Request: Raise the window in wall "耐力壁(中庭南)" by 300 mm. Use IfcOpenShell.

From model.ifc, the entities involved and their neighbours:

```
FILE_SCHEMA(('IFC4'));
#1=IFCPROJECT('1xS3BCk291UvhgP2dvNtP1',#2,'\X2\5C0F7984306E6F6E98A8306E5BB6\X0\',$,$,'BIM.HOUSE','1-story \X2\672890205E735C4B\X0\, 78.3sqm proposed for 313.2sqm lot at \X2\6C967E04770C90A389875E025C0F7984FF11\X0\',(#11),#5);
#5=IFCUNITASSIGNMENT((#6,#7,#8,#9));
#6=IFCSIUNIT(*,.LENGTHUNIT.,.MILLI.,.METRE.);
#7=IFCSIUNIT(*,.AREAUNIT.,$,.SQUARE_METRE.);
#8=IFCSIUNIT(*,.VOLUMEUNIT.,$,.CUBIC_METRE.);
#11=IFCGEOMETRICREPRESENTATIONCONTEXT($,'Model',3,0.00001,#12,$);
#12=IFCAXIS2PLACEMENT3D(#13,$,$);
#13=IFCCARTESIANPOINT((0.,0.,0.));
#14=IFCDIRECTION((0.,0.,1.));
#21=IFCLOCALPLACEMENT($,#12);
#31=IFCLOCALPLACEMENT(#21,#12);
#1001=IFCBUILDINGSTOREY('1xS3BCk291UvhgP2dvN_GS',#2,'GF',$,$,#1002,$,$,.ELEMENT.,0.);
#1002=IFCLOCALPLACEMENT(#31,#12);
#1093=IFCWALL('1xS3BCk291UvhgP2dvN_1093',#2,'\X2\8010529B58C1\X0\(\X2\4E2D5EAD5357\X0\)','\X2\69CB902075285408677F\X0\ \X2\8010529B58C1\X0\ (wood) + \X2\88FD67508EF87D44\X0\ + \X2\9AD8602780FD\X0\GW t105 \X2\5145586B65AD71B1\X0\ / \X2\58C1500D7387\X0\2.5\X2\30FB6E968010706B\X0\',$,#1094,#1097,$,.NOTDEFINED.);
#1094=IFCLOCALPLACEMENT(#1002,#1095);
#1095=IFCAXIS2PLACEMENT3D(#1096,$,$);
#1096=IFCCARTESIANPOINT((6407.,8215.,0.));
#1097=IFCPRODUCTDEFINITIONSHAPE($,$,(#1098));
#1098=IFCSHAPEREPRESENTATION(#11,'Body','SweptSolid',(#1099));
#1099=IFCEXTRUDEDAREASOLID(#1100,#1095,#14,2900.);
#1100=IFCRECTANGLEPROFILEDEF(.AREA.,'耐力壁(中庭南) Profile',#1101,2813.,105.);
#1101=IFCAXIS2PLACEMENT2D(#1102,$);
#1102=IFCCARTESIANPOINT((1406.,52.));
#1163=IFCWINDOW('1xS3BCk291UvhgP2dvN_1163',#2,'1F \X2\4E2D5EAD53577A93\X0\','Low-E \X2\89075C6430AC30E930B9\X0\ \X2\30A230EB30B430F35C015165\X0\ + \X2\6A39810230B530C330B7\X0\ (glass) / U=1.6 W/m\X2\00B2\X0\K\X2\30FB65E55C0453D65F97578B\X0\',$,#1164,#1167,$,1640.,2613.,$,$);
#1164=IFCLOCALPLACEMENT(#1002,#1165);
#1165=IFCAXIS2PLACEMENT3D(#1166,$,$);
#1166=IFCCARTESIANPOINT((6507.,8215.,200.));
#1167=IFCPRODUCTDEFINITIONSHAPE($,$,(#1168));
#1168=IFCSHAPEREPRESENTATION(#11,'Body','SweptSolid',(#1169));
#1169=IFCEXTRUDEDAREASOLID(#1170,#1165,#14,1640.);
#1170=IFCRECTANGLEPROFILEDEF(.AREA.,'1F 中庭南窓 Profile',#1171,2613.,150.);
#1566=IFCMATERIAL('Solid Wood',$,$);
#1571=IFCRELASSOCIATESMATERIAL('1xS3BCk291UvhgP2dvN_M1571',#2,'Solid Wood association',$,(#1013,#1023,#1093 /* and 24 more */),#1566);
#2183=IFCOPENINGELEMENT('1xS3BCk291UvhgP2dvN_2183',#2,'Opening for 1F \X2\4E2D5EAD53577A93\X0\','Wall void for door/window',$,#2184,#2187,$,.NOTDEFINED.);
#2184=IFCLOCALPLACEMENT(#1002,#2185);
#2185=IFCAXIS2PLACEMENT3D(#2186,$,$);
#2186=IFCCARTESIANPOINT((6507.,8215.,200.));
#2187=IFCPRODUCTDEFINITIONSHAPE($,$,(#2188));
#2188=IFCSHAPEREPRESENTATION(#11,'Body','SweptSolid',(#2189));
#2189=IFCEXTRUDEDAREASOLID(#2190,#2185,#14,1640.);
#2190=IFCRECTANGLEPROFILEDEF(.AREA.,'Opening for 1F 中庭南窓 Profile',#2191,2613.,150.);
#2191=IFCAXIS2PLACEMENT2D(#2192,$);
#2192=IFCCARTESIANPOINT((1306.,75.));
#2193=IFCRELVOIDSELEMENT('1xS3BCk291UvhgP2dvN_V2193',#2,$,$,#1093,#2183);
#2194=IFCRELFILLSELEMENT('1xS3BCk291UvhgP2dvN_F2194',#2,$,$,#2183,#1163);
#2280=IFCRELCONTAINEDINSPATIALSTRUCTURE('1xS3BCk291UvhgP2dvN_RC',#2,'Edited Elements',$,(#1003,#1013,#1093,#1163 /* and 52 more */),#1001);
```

```python
import numpy as np
import ifcopenshell
import ifcopenshell.api.geometry
import ifcopenshell.util.placement
import ifcopenshell.util.unit

model = ifcopenshell.open("model.ifc")
unit_scale = ifcopenshell.util.unit.calculate_unit_scale(model)

window = model.by_id(1163)
opening = window.FillsVoids[0].RelatingOpeningElement
dz = 300.0

shift = np.array([0.0, 0.0, dz])
# The window is not placed relative to its opening, so move both.
for product in (opening, window):
    matrix = ifcopenshell.util.placement.get_local_placement(product.ObjectPlacement)
    matrix[:3, 3] += shift
    ifcopenshell.api.geometry.edit_object_placement(model, product=product, matrix=matrix, is_si=False)

print(f"moved by {dz * unit_scale:+.3f} m")

model.write("model-out.ifc")
```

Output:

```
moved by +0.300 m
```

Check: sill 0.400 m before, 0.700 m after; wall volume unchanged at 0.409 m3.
